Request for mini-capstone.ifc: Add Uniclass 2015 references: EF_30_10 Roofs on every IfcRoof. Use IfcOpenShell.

First a look at what the model holds.

```python
import ifcopenshell

model = ifcopenshell.open("mini-capstone.ifc")
print(model.schema)
print("classifications:", [c.Name for c in model.by_type("IfcClassification")])
for ifc_class in ("IfcDoor", "IfcRoof", "IfcStair", "IfcWall", "IfcWindow"):
    print(ifc_class, len(model.by_type(ifc_class)))
```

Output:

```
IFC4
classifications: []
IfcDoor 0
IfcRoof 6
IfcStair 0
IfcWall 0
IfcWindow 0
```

```python
import ifcopenshell
import ifcopenshell.api.classification

model = ifcopenshell.open("mini-capstone.ifc")

system = ifcopenshell.api.classification.add_classification(model, classification="Uniclass 2015")

codes = {
    "IfcRoof": ("EF_30_10", "Roofs"),
}
for ifc_class, (code, name) in codes.items():
    products = model.by_type(ifc_class)
    ifcopenshell.api.classification.add_reference(
        model, products=products, classification=system, identification=code, name=name
    )
    print(code, len(products))

model.write("mini-capstone_rev.ifc")
```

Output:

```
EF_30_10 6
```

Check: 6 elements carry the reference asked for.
